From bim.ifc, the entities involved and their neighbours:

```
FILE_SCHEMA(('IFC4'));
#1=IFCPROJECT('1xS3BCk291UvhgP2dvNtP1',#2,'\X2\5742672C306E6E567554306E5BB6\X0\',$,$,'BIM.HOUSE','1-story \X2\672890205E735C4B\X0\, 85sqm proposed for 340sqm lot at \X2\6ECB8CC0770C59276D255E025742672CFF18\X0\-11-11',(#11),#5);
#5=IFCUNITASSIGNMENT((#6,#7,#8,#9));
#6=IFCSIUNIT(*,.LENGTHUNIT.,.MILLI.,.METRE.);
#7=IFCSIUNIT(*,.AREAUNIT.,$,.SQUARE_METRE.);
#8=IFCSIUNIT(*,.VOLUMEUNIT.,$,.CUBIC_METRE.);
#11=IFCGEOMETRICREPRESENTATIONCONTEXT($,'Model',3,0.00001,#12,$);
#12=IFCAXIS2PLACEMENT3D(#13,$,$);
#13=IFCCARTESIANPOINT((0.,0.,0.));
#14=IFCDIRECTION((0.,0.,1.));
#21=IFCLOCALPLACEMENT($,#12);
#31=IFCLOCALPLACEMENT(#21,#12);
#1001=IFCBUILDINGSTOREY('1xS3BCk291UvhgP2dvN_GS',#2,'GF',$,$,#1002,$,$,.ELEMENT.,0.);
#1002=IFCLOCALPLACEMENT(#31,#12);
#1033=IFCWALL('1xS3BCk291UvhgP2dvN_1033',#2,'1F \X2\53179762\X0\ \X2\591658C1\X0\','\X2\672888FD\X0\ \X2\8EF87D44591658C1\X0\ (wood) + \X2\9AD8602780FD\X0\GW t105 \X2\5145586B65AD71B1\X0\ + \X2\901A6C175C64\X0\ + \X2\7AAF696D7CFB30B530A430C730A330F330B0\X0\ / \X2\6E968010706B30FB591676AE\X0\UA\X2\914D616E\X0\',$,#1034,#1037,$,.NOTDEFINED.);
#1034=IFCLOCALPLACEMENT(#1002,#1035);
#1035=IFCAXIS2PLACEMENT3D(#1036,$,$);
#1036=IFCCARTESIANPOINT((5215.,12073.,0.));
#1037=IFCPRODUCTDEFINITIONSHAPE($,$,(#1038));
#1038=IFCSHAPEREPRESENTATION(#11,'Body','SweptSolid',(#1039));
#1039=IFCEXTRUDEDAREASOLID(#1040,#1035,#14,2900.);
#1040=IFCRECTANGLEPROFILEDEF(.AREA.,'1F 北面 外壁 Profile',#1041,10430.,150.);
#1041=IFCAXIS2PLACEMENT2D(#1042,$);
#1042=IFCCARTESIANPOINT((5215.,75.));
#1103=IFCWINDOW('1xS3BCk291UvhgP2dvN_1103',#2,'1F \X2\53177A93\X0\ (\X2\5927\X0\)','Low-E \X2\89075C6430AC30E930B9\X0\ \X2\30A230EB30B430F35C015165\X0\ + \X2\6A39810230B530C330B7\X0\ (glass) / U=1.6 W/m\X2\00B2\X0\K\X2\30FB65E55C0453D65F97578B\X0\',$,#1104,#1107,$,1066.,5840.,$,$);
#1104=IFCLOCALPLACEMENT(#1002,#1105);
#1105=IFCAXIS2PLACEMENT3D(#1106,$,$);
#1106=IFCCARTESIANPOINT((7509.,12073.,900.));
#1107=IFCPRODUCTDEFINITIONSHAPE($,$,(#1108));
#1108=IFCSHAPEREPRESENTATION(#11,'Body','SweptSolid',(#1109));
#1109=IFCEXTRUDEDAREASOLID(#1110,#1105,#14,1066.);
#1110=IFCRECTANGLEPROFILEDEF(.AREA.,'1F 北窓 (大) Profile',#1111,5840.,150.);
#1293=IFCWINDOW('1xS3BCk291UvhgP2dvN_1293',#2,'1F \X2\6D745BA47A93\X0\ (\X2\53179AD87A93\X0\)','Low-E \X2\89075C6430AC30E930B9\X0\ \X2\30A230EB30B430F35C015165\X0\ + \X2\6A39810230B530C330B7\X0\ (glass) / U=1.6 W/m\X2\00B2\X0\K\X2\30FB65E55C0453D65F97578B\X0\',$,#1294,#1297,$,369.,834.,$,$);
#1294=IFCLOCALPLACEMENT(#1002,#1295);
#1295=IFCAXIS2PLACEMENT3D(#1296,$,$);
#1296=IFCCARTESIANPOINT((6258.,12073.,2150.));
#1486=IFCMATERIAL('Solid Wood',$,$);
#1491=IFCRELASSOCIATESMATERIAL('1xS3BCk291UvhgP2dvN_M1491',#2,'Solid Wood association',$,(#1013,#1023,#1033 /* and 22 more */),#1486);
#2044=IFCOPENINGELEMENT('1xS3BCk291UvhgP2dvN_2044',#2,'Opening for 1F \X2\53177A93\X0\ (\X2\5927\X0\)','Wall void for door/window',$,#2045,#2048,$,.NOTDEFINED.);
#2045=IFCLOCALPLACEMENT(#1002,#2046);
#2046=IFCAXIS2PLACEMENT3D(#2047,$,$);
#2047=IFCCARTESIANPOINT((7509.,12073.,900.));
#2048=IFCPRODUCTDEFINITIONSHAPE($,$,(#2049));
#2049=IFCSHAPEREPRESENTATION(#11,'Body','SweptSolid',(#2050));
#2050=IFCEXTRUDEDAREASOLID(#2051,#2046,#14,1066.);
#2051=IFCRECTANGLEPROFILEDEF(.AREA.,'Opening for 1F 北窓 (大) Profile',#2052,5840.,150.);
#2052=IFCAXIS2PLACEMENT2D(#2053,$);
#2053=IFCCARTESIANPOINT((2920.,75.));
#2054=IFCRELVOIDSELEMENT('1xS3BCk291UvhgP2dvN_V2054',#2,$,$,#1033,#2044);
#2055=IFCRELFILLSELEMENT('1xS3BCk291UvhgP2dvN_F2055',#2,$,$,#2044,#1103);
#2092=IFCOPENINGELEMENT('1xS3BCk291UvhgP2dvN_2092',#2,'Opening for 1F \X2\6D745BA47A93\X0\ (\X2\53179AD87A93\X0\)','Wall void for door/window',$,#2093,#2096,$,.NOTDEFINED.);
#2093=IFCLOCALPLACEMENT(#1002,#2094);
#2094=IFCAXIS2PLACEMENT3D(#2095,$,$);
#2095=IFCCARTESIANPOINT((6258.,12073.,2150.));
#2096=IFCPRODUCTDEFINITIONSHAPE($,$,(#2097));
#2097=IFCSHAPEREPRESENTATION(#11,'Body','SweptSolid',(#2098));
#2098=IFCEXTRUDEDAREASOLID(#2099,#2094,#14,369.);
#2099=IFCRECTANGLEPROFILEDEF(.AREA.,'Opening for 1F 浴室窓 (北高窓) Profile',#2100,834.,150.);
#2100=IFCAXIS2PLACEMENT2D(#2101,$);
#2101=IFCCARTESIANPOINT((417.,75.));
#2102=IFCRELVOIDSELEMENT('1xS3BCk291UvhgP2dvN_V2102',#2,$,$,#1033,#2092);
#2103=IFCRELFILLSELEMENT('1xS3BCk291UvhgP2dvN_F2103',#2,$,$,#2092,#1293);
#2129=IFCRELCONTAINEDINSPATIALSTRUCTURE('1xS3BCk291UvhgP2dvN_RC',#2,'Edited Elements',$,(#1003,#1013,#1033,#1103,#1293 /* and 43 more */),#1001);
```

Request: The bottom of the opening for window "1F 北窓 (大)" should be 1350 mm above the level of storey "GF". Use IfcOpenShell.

```python
import numpy as np
import ifcopenshell
import ifcopenshell.api.geometry
import ifcopenshell.geom
import ifcopenshell.util.element
import ifcopenshell.util.placement
import ifcopenshell.util.shape
import ifcopenshell.util.unit

model = ifcopenshell.open("bim.ifc")
unit_scale = ifcopenshell.util.unit.calculate_unit_scale(model)

window = model.by_guid("1xS3BCk291UvhgP2dvN_1103")
opening = window.FillsVoids[0].RelatingOpeningElement
storey = ifcopenshell.util.element.get_container(window, ifc_class="IfcBuildingStorey")
level = ifcopenshell.util.placement.get_local_placement(storey.ObjectPlacement)[2, 3]

# The opening's origin need not be at the sill, so measure its lowest point.
shape = ifcopenshell.geom.create_shape(ifcopenshell.geom.settings(), opening)
bottom = ifcopenshell.util.shape.get_shape_bottom_elevation(shape, shape.geometry) / unit_scale
dz = level + 1350.0 - bottom

shift = np.array([0.0, 0.0, dz])
# The window is not placed relative to its opening, so move both.
for product in (opening, window):
    matrix = ifcopenshell.util.placement.get_local_placement(product.ObjectPlacement)
    matrix[:3, 3] += shift
    ifcopenshell.api.geometry.edit_object_placement(model, product=product, matrix=matrix, is_si=False)

print(f"moved by {dz * unit_scale:+.3f} m")

model.write("bim_edited.ifc")
```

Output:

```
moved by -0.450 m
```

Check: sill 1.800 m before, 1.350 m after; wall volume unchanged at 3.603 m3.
